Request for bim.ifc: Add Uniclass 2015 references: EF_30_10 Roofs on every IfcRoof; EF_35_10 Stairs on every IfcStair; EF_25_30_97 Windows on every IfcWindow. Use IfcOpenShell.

First a look at what the model holds.

```python
import ifcopenshell

model = ifcopenshell.open("bim.ifc")
print(model.schema)
print("classifications:", [c.Name for c in model.by_type("IfcClassification")])
for ifc_class in ("IfcDoor", "IfcRoof", "IfcStair", "IfcWall", "IfcWindow"):
    print(ifc_class, len(model.by_type(ifc_class)))
```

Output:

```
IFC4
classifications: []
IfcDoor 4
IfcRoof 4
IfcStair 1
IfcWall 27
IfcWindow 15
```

```python
import ifcopenshell
import ifcopenshell.api.classification

model = ifcopenshell.open("bim.ifc")

system = ifcopenshell.api.classification.add_classification(model, classification="Uniclass 2015")

codes = {
    "IfcRoof": ("EF_30_10", "Roofs"),
    "IfcStair": ("EF_35_10", "Stairs"),
    "IfcWindow": ("EF_25_30_97", "Windows"),
}
for ifc_class, (code, name) in codes.items():
    products = model.by_type(ifc_class)
    ifcopenshell.api.classification.add_reference(
        model, products=products, classification=system, identification=code, name=name
    )
    print(code, len(products))

model.write("bim_rev.ifc")
```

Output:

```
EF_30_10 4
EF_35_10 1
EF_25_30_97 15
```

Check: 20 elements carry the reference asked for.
